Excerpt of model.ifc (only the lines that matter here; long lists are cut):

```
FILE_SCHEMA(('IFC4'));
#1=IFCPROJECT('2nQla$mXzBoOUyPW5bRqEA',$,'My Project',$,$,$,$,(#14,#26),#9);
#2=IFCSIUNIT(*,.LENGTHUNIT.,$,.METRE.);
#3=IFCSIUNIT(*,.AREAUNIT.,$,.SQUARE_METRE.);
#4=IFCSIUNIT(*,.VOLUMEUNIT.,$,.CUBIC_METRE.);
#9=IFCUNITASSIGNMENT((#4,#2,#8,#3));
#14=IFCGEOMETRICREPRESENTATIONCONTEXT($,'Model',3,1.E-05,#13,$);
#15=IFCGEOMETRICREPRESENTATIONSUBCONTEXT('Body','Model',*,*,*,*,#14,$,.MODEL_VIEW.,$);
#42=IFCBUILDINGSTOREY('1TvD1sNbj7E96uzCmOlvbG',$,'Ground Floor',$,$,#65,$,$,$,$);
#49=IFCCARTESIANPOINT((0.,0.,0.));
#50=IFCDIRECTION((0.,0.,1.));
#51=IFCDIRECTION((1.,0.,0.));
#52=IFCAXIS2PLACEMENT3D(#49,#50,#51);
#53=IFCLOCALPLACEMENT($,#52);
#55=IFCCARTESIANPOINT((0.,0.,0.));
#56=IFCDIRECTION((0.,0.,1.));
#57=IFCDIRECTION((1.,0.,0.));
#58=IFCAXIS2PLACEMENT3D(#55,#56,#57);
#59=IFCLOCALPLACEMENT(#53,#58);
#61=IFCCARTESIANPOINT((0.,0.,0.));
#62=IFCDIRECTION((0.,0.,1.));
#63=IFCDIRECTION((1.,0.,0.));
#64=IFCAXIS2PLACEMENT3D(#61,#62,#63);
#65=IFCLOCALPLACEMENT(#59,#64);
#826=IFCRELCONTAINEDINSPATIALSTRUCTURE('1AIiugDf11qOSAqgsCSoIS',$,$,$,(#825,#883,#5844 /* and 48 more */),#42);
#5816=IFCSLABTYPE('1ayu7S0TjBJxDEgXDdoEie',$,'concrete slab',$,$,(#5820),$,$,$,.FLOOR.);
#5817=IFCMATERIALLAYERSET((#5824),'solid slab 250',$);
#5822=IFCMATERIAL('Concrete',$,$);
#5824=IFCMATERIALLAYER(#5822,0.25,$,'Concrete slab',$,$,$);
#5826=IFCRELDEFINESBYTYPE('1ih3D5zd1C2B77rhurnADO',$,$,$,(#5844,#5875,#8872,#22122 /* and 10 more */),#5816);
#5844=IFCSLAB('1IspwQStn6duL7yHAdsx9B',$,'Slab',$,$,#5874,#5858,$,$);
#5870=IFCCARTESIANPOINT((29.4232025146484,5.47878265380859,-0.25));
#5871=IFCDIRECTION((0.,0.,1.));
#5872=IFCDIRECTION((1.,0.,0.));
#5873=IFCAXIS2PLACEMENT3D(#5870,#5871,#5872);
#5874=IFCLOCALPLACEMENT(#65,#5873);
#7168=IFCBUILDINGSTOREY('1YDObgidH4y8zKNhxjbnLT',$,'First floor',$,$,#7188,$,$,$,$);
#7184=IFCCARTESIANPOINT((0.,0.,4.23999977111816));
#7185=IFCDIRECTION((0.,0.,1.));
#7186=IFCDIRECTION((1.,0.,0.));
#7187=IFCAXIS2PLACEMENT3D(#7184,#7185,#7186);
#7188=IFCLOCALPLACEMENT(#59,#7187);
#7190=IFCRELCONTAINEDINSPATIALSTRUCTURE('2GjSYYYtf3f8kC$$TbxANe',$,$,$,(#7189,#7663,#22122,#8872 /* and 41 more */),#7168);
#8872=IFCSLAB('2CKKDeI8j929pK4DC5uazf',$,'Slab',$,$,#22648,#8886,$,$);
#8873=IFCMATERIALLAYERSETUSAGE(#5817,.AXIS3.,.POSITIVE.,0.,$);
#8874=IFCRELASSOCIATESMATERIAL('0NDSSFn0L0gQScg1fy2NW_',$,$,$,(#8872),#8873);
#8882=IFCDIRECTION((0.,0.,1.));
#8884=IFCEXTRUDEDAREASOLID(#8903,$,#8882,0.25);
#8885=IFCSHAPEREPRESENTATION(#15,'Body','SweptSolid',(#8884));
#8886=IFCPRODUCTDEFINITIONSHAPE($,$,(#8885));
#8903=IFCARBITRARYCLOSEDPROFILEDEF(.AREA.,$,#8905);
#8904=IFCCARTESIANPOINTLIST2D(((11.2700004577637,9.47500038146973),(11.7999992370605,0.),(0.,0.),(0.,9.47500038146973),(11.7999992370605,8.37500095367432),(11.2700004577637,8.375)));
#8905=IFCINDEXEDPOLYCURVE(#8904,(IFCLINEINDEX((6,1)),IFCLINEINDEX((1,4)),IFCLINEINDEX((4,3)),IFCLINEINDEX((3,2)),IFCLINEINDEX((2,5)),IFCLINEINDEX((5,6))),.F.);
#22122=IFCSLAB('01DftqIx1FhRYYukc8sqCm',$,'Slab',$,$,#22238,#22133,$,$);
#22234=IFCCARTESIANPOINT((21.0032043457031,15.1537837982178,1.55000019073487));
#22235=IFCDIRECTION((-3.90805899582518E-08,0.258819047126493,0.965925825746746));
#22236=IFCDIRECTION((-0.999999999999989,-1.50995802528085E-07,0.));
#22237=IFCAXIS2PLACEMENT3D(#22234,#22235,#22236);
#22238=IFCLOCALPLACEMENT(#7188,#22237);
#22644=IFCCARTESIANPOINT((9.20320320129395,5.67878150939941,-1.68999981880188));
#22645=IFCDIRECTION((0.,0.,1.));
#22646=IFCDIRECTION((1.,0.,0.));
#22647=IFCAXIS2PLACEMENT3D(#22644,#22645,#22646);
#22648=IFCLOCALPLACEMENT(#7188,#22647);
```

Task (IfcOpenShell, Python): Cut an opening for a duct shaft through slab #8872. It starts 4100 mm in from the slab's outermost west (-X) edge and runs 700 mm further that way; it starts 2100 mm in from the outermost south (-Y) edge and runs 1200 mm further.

```python
import numpy as np
import ifcopenshell
import ifcopenshell.api.feature
import ifcopenshell.api.geometry
import ifcopenshell.api.root
import ifcopenshell.geom
import ifcopenshell.util.placement
import ifcopenshell.util.representation
import ifcopenshell.util.shape
import ifcopenshell.util.unit

model = ifcopenshell.open("model.ifc")
unit_scale = ifcopenshell.util.unit.calculate_unit_scale(model)
settings = ifcopenshell.geom.settings()


def volume(element):
    """Net volume in cubic metres, openings subtracted."""
    shape = ifcopenshell.geom.create_shape(settings, element)
    return ifcopenshell.util.shape.get_volume(shape.geometry)


slab = model.by_id(8872)
before = volume(slab)

# Extent in the slab's own axes, in metres. The edges named are its -X and -Y sides.
slab_shape = ifcopenshell.geom.create_shape(settings, slab)
vertices = ifcopenshell.util.shape.get_vertices(slab_shape.geometry)
x_min, y_min, bottom = vertices.min(axis=0)
top = vertices[:, 2].max()

opening = ifcopenshell.api.root.create_entity(model, ifc_class="IfcOpeningElement", name="Duct shaft opening", predefined_type="OPENING")
context = ifcopenshell.util.representation.get_context(model, "Model", "Body", "MODEL_VIEW")
width, depth = 0.7, 1.2
outline = [(0.0, 0.0), (width, 0.0), (width, depth), (0.0, depth), (0.0, 0.0)]
# Overshoot both faces by 50 mm so the cut is clean.
shape = ifcopenshell.api.geometry.add_slab_representation(
    model, context=context, depth=top - bottom + 0.1, polyline=outline
)
ifcopenshell.api.geometry.assign_representation(model, product=opening, representation=shape)

matrix = ifcopenshell.util.placement.get_local_placement(slab.ObjectPlacement)
matrix[:, 3] = matrix @ np.append(np.array([x_min + 4.1, y_min + 2.1, bottom - 0.05]) / unit_scale, 1.0)
ifcopenshell.api.geometry.edit_object_placement(model, product=opening, matrix=matrix, is_si=False)
ifcopenshell.api.feature.add_feature(model, feature=opening, element=slab)

after = volume(slab)

print(f"slab volume {before:.3f} -> {after:.3f} m3")

model.write("model_updated.ifc")
```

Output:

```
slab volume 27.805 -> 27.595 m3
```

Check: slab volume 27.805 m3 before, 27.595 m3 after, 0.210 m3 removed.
